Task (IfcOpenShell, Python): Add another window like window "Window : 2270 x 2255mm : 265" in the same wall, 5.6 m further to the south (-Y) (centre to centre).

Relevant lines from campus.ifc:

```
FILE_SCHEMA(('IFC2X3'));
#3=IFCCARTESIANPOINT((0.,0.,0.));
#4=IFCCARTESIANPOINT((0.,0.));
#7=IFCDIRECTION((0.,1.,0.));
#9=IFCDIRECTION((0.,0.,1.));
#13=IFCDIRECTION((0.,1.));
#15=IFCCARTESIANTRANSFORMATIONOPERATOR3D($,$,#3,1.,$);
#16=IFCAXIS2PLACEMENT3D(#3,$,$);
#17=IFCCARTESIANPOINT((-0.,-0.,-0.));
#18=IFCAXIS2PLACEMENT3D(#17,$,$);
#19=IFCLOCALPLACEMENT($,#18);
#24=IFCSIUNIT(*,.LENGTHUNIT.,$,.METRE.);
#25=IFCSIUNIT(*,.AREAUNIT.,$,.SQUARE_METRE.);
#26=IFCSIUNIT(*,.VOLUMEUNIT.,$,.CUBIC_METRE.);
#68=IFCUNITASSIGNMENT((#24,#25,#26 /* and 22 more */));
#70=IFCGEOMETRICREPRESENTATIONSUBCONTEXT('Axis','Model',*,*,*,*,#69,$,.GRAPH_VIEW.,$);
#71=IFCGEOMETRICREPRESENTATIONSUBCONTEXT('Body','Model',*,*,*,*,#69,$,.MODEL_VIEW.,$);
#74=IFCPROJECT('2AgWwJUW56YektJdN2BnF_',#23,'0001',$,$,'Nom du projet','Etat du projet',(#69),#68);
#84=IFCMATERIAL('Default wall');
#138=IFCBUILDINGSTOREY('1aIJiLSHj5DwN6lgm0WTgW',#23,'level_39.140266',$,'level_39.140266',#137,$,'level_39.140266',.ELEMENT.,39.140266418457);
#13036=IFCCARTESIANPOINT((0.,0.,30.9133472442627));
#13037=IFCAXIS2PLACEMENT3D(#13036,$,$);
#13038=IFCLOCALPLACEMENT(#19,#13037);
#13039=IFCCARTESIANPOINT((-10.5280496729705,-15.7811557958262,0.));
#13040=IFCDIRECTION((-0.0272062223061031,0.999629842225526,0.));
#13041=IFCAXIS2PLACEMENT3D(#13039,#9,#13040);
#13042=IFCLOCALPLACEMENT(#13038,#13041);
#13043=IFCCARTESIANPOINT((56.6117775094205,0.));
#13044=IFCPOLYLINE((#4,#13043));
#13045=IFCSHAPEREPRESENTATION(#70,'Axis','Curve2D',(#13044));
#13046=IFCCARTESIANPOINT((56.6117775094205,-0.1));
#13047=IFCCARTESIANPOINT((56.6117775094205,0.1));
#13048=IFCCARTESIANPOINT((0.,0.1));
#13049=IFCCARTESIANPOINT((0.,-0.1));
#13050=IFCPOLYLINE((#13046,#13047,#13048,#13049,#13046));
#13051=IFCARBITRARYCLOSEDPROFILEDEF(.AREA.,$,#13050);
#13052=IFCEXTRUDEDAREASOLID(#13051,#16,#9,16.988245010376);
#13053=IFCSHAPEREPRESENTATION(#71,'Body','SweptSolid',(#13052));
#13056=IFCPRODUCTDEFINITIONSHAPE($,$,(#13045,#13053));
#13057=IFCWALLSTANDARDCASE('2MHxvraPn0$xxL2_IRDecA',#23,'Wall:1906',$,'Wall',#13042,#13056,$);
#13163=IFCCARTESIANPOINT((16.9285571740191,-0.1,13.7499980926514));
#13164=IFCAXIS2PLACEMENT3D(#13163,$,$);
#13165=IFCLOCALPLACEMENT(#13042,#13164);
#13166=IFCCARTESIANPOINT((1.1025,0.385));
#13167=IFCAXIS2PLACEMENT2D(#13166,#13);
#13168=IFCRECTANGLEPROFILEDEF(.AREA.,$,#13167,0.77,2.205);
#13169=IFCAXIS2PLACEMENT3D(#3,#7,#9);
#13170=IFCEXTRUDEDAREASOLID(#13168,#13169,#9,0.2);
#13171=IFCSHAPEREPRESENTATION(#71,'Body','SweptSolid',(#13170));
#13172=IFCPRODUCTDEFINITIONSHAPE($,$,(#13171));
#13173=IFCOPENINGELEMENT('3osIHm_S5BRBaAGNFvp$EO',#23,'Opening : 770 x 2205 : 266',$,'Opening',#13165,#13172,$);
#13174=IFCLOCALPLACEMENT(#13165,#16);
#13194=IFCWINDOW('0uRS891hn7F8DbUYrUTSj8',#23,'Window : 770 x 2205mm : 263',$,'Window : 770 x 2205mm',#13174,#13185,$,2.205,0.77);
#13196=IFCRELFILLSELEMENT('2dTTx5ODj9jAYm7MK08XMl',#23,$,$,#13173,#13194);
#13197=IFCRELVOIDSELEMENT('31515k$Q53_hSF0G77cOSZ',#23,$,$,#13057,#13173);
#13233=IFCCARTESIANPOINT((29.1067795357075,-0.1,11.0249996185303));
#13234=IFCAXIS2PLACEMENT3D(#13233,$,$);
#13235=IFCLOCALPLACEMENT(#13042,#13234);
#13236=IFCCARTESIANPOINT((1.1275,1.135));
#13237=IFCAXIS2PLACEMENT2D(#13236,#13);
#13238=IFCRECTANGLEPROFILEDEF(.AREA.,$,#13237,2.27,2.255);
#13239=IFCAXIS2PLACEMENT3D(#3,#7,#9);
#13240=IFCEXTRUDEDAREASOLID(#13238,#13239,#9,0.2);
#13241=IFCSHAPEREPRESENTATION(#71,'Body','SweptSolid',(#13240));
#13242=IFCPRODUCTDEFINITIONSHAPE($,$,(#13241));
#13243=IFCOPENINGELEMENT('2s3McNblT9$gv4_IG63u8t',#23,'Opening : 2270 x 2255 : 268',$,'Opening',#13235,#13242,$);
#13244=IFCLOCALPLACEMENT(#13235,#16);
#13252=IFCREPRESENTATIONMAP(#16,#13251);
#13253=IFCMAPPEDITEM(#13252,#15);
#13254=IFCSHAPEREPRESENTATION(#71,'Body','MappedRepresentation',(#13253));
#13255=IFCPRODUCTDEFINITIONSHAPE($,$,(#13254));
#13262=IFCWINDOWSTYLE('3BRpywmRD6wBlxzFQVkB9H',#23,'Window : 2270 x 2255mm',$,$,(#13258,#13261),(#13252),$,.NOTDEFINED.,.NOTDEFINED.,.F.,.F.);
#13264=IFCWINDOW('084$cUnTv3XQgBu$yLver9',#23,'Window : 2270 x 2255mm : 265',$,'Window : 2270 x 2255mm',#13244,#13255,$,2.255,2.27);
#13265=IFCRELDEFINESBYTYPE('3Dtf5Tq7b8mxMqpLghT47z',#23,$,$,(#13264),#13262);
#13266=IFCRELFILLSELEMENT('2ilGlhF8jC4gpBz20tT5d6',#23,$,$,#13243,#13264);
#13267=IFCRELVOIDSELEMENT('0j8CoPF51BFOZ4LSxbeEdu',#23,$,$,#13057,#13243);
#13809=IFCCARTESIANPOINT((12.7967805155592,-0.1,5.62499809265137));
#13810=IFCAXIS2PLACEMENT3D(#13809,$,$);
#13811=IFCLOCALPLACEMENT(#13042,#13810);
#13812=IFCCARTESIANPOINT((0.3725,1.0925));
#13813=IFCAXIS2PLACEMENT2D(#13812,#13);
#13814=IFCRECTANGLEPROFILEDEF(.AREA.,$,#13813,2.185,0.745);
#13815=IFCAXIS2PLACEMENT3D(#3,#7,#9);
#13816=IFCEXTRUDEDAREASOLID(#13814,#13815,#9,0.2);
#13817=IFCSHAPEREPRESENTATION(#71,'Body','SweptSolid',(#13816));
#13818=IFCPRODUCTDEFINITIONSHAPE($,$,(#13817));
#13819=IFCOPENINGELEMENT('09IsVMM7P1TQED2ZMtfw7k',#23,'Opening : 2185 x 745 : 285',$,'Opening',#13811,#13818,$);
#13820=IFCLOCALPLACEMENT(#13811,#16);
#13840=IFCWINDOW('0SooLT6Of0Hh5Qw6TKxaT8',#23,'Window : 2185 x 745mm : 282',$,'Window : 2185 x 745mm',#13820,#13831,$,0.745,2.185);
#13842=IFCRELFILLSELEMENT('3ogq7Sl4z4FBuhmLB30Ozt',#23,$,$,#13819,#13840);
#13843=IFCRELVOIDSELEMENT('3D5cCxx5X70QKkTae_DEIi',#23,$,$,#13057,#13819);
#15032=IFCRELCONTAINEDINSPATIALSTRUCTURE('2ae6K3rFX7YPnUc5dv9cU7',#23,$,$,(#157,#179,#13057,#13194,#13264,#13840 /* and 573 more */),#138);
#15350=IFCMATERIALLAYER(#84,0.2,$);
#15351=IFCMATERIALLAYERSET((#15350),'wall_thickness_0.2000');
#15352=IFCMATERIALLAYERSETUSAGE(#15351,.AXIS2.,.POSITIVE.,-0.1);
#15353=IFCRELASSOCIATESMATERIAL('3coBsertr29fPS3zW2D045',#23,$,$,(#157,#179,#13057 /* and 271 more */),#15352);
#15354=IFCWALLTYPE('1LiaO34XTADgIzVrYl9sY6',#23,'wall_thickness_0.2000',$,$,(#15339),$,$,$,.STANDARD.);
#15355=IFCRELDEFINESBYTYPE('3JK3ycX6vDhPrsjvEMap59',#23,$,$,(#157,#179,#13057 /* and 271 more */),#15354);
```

```python
import ifcopenshell
import ifcopenshell.api.feature
import ifcopenshell.api.geometry
import ifcopenshell.api.root
import ifcopenshell.geom
import ifcopenshell.util.element
import ifcopenshell.util.placement
import ifcopenshell.util.shape
import ifcopenshell.util.unit

model = ifcopenshell.open("campus.ifc")
unit_scale = ifcopenshell.util.unit.calculate_unit_scale(model)
settings = ifcopenshell.geom.settings()


def volume(element):
    """Net volume in cubic metres, openings subtracted."""
    shape = ifcopenshell.geom.create_shape(settings, element)
    return ifcopenshell.util.shape.get_volume(shape.geometry)


window = model.by_guid("084$cUnTv3XQgBu$yLver9")
opening = window.FillsVoids[0].RelatingOpeningElement
wall = opening.VoidsElements[0].RelatingBuildingElement
before = volume(wall)
shift = ifcopenshell.util.placement.get_local_placement(wall.ObjectPlacement)[:3, 0] * -5.6 / unit_scale

# copy_class copies the void relationship, type, container and properties, but no geometry.
new_opening = ifcopenshell.api.root.copy_class(model, product=opening)
new_opening.Representation = ifcopenshell.util.element.copy_deep(
    model, opening.Representation, exclude=["IfcGeometricRepresentationContext", "IfcRepresentationMap"]
)
new_opening.Name = "Opening : 2270 x 2255"
new_window = ifcopenshell.api.root.copy_class(model, product=window)
new_window.Representation = ifcopenshell.util.element.copy_deep(
    model, window.Representation, exclude=["IfcGeometricRepresentationContext", "IfcRepresentationMap"]
)
new_window.Name = "Window : 2270 x 2255mm"
fills = ifcopenshell.api.feature.add_filling(model, opening=new_opening, element=new_window)
fills.OwnerHistory = new_window.OwnerHistory  # required in IFC2X3

for old, new in ((opening, new_opening), (window, new_window)):
    matrix = ifcopenshell.util.placement.get_local_placement(old.ObjectPlacement)
    matrix[:3, 3] += shift
    ifcopenshell.api.geometry.edit_object_placement(model, product=new, matrix=matrix, is_si=False)

after = volume(wall)

print(f"wall volume {before:.3f} -> {after:.3f} m3")

model.write("campus_v2.ifc")
```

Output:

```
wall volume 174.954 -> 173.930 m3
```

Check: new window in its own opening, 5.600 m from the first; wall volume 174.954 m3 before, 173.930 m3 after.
